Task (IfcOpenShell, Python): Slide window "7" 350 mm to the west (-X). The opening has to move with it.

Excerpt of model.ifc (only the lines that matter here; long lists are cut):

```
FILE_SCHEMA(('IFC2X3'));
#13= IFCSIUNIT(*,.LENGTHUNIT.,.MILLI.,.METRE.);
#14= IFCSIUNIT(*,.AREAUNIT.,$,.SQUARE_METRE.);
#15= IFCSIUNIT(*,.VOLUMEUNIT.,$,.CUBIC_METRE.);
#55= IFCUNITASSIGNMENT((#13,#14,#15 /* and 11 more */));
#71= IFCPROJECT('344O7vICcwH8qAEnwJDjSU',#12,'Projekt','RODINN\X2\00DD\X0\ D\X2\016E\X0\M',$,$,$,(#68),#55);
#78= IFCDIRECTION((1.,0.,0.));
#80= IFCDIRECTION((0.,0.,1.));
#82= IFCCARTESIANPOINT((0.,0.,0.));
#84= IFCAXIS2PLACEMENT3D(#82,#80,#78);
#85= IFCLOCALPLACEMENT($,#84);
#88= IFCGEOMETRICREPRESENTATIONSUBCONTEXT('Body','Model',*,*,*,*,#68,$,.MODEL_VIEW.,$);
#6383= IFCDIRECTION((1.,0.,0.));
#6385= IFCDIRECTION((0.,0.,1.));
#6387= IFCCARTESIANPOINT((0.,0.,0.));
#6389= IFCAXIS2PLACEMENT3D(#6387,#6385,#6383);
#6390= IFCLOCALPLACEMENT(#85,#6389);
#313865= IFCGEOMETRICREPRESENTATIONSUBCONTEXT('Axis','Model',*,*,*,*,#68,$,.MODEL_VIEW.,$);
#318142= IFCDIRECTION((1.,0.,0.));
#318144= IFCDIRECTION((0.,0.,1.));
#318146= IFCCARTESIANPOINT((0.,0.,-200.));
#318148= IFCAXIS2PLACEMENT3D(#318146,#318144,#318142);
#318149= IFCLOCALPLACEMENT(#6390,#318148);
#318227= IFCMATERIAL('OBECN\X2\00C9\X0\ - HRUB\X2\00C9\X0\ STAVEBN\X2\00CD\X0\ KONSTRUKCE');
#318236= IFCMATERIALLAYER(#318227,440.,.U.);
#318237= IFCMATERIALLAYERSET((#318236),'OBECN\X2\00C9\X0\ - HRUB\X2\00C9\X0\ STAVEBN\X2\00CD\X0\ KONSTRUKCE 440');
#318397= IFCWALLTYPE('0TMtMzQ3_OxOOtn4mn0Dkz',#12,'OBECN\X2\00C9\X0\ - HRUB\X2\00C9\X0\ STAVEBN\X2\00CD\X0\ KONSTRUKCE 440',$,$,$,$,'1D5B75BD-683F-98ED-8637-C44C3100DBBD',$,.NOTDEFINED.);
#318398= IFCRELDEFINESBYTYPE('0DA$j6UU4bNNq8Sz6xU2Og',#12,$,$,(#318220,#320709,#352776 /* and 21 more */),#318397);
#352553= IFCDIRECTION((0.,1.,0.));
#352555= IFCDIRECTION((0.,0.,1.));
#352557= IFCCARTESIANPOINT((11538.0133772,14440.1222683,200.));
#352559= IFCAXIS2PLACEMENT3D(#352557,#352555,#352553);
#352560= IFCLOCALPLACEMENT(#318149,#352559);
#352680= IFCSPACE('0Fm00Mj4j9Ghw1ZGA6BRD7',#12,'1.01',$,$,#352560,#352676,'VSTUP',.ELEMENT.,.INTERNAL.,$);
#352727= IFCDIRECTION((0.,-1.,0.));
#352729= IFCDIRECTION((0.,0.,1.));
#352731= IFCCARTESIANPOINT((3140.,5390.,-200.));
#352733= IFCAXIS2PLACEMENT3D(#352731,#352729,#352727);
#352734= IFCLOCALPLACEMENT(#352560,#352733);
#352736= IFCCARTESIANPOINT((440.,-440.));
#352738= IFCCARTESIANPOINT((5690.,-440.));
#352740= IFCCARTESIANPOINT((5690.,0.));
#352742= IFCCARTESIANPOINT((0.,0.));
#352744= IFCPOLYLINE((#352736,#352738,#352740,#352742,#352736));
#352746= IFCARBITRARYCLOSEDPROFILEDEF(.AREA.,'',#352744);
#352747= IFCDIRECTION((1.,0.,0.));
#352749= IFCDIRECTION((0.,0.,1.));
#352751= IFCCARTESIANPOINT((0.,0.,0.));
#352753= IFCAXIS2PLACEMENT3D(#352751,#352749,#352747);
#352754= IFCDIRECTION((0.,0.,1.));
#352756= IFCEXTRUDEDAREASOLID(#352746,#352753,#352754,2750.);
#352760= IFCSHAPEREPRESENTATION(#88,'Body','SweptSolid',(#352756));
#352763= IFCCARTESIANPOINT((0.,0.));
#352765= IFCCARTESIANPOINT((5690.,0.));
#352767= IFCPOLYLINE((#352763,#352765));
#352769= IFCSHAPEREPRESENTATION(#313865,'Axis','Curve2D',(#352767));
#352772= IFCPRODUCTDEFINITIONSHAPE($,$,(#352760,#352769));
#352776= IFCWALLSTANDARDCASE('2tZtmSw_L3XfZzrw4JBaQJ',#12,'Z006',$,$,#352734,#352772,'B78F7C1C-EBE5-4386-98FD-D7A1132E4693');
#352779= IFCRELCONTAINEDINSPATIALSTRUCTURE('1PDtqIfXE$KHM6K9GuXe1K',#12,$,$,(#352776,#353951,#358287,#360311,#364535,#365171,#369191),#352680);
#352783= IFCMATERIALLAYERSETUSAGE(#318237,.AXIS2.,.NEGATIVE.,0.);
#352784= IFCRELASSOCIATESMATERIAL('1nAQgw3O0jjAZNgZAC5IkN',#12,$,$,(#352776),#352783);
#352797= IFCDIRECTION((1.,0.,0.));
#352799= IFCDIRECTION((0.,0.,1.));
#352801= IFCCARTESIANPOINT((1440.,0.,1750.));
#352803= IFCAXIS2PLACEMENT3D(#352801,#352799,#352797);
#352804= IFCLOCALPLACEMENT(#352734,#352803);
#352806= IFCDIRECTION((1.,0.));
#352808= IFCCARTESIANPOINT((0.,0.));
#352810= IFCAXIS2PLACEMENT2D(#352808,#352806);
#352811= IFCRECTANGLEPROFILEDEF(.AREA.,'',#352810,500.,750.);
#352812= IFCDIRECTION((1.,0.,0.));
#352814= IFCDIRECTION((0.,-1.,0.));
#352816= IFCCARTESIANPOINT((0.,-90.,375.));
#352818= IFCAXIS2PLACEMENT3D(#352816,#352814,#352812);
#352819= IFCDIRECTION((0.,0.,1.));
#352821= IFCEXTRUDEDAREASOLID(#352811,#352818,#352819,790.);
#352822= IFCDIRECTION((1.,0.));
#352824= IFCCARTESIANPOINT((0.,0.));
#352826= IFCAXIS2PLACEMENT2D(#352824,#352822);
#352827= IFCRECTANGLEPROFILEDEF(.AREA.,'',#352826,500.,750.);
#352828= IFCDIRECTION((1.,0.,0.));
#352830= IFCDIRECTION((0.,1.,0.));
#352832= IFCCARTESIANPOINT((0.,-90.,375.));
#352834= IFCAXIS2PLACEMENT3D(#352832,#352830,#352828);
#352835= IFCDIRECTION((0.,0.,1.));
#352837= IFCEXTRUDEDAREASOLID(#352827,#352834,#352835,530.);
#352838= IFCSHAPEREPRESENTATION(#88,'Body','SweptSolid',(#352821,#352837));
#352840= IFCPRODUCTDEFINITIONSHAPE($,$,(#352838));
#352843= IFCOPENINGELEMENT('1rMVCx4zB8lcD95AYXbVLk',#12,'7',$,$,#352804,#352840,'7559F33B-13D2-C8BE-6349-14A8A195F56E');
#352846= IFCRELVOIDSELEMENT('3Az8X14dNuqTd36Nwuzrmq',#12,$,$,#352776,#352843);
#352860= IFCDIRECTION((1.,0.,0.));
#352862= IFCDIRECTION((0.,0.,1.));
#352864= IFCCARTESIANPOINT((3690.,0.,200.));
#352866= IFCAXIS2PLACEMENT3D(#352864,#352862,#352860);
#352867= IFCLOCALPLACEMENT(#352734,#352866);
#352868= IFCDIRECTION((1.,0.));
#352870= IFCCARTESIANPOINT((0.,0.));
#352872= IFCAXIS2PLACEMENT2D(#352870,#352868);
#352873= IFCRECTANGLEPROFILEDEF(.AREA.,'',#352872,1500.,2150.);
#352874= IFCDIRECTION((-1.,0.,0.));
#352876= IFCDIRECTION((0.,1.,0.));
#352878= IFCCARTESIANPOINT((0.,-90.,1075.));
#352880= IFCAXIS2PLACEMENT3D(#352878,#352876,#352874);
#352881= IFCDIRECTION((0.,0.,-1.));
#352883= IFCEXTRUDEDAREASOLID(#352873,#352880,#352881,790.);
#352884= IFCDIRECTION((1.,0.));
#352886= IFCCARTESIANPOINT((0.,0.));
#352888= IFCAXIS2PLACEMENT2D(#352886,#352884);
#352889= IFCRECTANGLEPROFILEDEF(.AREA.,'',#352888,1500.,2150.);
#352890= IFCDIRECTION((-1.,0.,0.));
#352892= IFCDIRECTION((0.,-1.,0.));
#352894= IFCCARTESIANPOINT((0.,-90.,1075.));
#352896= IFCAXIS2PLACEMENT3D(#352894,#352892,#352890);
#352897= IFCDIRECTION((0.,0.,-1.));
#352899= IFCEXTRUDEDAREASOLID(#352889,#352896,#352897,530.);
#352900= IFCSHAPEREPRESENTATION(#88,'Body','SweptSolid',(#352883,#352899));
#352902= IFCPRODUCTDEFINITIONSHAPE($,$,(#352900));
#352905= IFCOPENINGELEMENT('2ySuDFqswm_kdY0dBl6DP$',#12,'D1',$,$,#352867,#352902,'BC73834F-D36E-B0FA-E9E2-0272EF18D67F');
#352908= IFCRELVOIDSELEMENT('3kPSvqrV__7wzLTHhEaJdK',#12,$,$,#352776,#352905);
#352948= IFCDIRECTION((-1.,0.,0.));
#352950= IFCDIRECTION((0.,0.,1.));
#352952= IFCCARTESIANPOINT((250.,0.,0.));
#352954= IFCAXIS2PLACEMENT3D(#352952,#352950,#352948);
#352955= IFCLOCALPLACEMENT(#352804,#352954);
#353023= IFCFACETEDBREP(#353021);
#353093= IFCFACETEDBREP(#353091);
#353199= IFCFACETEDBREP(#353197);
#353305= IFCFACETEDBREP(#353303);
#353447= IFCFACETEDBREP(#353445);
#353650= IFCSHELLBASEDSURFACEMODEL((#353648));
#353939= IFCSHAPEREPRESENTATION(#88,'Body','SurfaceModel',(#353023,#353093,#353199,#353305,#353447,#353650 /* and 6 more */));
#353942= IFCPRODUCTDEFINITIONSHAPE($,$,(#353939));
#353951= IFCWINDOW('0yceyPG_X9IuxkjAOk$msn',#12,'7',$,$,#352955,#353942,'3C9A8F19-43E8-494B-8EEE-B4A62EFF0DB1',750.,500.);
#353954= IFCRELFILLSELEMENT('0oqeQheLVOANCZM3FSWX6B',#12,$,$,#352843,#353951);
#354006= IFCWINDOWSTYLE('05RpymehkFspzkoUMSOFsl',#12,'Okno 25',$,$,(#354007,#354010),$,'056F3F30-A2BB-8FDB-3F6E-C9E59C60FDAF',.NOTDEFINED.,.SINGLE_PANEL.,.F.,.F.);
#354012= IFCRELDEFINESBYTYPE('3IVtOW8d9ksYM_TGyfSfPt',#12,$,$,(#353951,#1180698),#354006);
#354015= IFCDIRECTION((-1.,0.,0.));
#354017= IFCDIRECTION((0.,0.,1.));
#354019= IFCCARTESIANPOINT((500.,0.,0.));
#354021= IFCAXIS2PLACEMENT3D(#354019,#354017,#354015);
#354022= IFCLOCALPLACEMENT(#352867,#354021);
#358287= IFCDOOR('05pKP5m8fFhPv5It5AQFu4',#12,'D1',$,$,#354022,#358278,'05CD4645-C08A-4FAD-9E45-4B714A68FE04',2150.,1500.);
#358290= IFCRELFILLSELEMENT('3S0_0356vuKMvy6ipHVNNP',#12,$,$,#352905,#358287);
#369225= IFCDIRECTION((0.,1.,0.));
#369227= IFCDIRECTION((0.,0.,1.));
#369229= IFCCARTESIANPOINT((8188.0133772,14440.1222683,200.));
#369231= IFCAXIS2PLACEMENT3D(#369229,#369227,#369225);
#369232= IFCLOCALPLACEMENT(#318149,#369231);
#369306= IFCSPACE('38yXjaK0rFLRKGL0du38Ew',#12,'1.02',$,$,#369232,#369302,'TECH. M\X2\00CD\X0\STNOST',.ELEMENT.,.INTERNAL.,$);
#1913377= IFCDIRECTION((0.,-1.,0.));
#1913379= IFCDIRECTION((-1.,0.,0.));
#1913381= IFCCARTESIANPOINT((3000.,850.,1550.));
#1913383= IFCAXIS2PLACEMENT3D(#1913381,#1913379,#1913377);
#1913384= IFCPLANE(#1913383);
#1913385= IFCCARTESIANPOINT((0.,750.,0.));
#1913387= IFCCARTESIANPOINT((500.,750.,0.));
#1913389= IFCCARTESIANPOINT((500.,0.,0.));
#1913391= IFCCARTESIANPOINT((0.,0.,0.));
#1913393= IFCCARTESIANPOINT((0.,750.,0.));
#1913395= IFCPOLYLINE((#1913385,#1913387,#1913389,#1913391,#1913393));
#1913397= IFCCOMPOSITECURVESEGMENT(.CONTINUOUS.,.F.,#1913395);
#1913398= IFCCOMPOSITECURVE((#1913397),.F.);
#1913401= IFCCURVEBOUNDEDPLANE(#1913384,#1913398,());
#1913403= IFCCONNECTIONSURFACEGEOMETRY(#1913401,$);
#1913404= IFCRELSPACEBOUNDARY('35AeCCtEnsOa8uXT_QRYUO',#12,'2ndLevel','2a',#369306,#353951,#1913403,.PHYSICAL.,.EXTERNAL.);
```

```python
import numpy as np
import ifcopenshell
import ifcopenshell.api.geometry
import ifcopenshell.util.placement
import ifcopenshell.util.unit

model = ifcopenshell.open("model.ifc")
unit_scale = ifcopenshell.util.unit.calculate_unit_scale(model)

window = model.by_guid("0yceyPG_X9IuxkjAOk$msn")
opening = window.FillsVoids[0].RelatingOpeningElement
wall = opening.VoidsElements[0].RelatingBuildingElement

wall_matrix = ifcopenshell.util.placement.get_local_placement(wall.ObjectPlacement)
shift = wall_matrix[:3, 0] * -0.35 / unit_scale
before = ifcopenshell.util.placement.get_local_placement(window.ObjectPlacement)[:3, 3].copy()

# The window is placed relative to its opening, so it follows when the opening moves.
matrix = ifcopenshell.util.placement.get_local_placement(opening.ObjectPlacement)
matrix[:3, 3] += shift
ifcopenshell.api.geometry.edit_object_placement(
    model, product=opening, matrix=matrix, is_si=False, should_transform_children=True
)

# Space boundary surfaces are stored in each space's coordinates; move them too.
for rel in window.ProvidesBoundaries:
    if not rel.ConnectionGeometry:
        continue
    surface = rel.ConnectionGeometry.SurfaceOnRelatingElement.BasisSurface
    space_matrix = ifcopenshell.util.placement.get_local_placement(rel.RelatingSpace.ObjectPlacement)
    point = np.array(surface.Position.Location.Coordinates) + space_matrix[:3, :3].T @ shift
    surface.Position = model.createIfcAxis2Placement3D(
        model.createIfcCartesianPoint(point.tolist()), surface.Position.Axis, surface.Position.RefDirection
    )

after = ifcopenshell.util.placement.get_local_placement(window.ObjectPlacement)[:3, 3]
print("window moved by", (after - before).round(3) + 0.0)

model.write("model-out.ifc")
```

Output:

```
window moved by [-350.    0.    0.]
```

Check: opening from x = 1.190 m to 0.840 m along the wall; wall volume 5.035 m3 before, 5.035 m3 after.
